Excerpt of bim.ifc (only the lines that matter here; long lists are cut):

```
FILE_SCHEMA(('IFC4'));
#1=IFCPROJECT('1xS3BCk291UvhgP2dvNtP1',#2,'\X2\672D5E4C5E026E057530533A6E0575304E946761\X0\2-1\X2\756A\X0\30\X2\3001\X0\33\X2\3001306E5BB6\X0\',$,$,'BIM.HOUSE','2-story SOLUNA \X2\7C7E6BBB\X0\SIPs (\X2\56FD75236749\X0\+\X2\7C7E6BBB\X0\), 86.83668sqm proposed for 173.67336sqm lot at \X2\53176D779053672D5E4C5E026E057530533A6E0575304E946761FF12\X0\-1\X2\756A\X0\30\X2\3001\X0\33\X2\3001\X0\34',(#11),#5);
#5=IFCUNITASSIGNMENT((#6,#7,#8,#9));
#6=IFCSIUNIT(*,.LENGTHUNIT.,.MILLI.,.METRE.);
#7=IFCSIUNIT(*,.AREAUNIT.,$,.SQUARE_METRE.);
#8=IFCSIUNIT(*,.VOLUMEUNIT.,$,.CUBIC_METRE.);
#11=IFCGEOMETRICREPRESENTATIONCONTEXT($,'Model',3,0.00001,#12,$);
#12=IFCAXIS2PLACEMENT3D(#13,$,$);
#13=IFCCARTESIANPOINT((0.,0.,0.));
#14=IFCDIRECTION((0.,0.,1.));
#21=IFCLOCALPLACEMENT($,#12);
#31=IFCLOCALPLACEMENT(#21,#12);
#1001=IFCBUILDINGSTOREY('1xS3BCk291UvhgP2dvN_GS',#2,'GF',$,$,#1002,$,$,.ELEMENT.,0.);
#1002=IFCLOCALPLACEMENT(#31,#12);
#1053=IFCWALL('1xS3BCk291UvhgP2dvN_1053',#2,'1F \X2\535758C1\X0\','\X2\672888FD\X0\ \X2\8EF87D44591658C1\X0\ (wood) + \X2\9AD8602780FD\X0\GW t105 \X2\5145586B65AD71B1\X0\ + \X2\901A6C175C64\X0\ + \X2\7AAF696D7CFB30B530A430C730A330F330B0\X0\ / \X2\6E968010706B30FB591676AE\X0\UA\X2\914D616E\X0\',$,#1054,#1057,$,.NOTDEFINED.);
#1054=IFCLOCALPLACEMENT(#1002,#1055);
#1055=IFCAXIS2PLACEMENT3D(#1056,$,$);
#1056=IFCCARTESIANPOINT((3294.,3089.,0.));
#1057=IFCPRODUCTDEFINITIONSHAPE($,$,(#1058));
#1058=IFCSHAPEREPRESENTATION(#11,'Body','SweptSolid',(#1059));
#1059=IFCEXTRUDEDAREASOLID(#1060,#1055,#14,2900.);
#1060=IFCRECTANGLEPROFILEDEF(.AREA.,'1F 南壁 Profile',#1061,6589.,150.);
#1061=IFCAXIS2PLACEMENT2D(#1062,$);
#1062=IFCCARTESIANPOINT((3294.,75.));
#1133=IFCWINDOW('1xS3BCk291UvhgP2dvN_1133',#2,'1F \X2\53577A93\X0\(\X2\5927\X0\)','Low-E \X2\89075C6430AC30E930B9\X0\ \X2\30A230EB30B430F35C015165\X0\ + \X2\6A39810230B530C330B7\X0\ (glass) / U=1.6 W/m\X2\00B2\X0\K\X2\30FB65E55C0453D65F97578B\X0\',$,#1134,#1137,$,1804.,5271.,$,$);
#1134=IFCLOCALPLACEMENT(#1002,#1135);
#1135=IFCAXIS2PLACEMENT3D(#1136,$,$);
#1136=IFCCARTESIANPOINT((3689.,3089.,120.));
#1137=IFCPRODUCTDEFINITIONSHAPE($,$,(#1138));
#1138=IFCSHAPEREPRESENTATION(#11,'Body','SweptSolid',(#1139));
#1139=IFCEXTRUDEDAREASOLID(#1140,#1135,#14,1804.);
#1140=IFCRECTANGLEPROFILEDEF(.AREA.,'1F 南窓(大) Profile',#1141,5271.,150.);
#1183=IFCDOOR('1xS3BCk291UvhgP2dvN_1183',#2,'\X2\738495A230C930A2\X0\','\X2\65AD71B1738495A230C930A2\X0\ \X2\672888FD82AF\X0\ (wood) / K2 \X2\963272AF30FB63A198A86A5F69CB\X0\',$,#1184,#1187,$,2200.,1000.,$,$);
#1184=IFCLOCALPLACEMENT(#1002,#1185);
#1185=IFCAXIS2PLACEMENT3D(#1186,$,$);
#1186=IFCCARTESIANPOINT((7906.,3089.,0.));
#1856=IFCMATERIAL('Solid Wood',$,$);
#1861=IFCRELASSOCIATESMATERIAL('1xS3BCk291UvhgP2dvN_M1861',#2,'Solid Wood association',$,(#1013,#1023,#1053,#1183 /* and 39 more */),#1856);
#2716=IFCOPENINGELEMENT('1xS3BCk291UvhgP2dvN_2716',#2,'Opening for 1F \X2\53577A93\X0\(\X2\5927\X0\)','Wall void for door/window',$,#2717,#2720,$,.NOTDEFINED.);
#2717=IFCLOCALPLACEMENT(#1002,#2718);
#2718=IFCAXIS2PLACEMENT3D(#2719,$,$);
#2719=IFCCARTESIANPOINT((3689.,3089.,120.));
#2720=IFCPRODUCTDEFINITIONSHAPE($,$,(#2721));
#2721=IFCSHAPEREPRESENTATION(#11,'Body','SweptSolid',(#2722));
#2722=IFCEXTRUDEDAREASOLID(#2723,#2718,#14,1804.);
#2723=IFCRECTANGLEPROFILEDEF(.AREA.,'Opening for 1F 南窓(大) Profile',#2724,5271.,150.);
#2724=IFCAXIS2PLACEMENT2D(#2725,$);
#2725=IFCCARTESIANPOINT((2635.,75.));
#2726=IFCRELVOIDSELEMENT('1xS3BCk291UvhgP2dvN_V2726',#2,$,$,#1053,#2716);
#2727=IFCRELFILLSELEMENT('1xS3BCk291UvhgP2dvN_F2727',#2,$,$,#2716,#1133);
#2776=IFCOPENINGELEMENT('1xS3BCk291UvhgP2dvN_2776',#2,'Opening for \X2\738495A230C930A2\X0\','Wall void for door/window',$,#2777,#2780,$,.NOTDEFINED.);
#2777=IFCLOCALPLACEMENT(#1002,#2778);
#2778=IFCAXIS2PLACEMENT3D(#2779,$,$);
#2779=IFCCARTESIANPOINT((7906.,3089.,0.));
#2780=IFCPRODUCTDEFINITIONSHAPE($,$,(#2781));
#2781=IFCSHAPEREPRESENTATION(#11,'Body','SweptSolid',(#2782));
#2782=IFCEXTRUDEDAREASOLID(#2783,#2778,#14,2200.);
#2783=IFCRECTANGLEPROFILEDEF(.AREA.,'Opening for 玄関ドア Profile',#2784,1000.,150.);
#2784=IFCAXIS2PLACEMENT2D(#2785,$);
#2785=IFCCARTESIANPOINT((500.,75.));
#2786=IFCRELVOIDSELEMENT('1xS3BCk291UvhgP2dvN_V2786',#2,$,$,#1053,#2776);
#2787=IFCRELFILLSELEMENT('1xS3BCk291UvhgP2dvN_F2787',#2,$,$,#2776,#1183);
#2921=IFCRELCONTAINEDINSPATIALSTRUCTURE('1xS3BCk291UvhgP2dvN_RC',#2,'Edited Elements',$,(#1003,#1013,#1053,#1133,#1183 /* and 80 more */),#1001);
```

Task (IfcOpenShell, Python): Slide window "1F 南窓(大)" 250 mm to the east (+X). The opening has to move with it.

```python
import ifcopenshell
import ifcopenshell.api.geometry
import ifcopenshell.util.placement
import ifcopenshell.util.unit

model = ifcopenshell.open("bim.ifc")
unit_scale = ifcopenshell.util.unit.calculate_unit_scale(model)

window = model.by_guid("1xS3BCk291UvhgP2dvN_1133")
opening = window.FillsVoids[0].RelatingOpeningElement
wall = opening.VoidsElements[0].RelatingBuildingElement

wall_matrix = ifcopenshell.util.placement.get_local_placement(wall.ObjectPlacement)
shift = wall_matrix[:3, 0] * 0.25 / unit_scale
before = ifcopenshell.util.placement.get_local_placement(window.ObjectPlacement)[:3, 3].copy()

# The window is not placed relative to its opening, so move both.
for product in (opening, window):
    matrix = ifcopenshell.util.placement.get_local_placement(product.ObjectPlacement)
    matrix[:3, 3] += shift
    ifcopenshell.api.geometry.edit_object_placement(model, product=product, matrix=matrix, is_si=False)

after = ifcopenshell.util.placement.get_local_placement(window.ObjectPlacement)[:3, 3]
print("window moved by", (after - before).round(3) + 0.0)

model.write("bim_v2.ifc")
```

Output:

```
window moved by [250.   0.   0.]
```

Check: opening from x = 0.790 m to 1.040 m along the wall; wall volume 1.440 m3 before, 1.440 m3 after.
